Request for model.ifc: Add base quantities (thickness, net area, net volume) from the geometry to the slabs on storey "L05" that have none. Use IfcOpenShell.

First a look at what the model holds.

```python
import ifcopenshell
import ifcopenshell.util.element
import ifcopenshell.util.unit

model = ifcopenshell.open("model.ifc")
print(model.schema)
for unit_type in ("LENGTHUNIT", "AREAUNIT", "VOLUMEUNIT"):
    print(unit_type, ifcopenshell.util.unit.calculate_unit_scale(model, unit_type))
storey = next(s for s in model.by_type("IfcBuildingStorey") if s.Name == "L05")
slabs = [e for e in ifcopenshell.util.element.get_decomposition(storey) if e.is_a("IfcSlab")]
for e in sorted(slabs, key=lambda e: e.id()):
    print(e.id(), e.is_a(), e.Name, list(ifcopenshell.util.element.get_psets(e, qtos_only=True)), sep=" | ")
```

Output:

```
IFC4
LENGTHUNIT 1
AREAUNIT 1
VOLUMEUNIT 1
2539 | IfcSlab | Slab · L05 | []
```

```python
import ifcopenshell
import ifcopenshell.api.pset
import ifcopenshell.geom
import ifcopenshell.util.element
import ifcopenshell.util.shape
import ifcopenshell.util.unit

model = ifcopenshell.open("model.ifc")
unit_scale = ifcopenshell.util.unit.calculate_unit_scale(model)
area_scale = ifcopenshell.util.unit.calculate_unit_scale(model, "AREAUNIT")
volume_scale = ifcopenshell.util.unit.calculate_unit_scale(model, "VOLUMEUNIT")
settings = ifcopenshell.geom.settings()

storey = next(s for s in model.by_type("IfcBuildingStorey") if s.Name == "L05")
slabs = [e for e in ifcopenshell.util.element.get_decomposition(storey) if e.is_a("IfcSlab")]

for e in sorted(slabs, key=lambda e: e.id()):
    if ifcopenshell.util.element.get_psets(e, qtos_only=True, should_inherit=False):
        continue
    # Geometry comes back in metres, in the element's own axes.
    shape = ifcopenshell.geom.create_shape(settings, e)
    values = {
        "Width": ifcopenshell.util.shape.get_z(shape.geometry) / unit_scale,
        "NetArea": ifcopenshell.util.shape.get_footprint_area(shape.geometry) / area_scale,
        "NetVolume": ifcopenshell.util.shape.get_volume(shape.geometry) / volume_scale,
    }
    qto = ifcopenshell.api.pset.add_qto(model, product=e, name="Qto_SlabBaseQuantities")
    ifcopenshell.api.pset.edit_qto(model, qto=qto, properties=values)
    print(e.id(), {k: round(v, 3) for k, v in values.items()})

model.write("model_rev.ifc")
```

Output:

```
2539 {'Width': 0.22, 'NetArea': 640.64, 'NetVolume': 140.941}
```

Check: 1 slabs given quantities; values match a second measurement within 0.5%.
